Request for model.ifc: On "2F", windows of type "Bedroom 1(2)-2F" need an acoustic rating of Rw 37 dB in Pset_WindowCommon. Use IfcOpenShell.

First a look at what the model holds.

```python
import ifcopenshell
import ifcopenshell.util.element

model = ifcopenshell.open("model.ifc")
print(model.schema)
storey = next(s for s in model.by_type("IfcBuildingStorey") if s.Name == "2F")
windows = [e for e in ifcopenshell.util.element.get_decomposition(storey) if e.is_a("IfcWindow")]
seen = {}
for e in windows:
    element_type = ifcopenshell.util.element.get_type(e)
    key = (element_type.Name if element_type != e and element_type else None, ifcopenshell.util.element.get_pset(e, "Pset_WindowCommon", "AcousticRating"))
    seen[key] = seen.get(key, 0) + 1
for (name, value), count in sorted(seen.items(), key=str):
    print(count, "x", name, "|", value)
```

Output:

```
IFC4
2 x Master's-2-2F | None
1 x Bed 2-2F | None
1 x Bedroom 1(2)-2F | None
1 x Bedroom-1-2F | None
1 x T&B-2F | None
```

```python
import ifcopenshell
import ifcopenshell.api.pset
import ifcopenshell.util.element

model = ifcopenshell.open("model.ifc")

storey = next(s for s in model.by_type("IfcBuildingStorey") if s.Name == "2F")
windows = [e for e in ifcopenshell.util.element.get_decomposition(storey) if e.is_a("IfcWindow")]

count = 0
for e in windows:
    element_type = ifcopenshell.util.element.get_type(e)
    if element_type in (None, e) or element_type.Name != "Bedroom 1(2)-2F":
        continue
    # add_pset returns the element's existing set when there is one.
    pset = ifcopenshell.api.pset.add_pset(model, product=e, name="Pset_WindowCommon")
    ifcopenshell.api.pset.edit_pset(model, pset=pset, properties={"AcousticRating": "Rw 37 dB"})
    count += 1

print(count, "windows updated")

model.write("model-out.ifc")
```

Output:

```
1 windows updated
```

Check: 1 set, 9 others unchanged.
